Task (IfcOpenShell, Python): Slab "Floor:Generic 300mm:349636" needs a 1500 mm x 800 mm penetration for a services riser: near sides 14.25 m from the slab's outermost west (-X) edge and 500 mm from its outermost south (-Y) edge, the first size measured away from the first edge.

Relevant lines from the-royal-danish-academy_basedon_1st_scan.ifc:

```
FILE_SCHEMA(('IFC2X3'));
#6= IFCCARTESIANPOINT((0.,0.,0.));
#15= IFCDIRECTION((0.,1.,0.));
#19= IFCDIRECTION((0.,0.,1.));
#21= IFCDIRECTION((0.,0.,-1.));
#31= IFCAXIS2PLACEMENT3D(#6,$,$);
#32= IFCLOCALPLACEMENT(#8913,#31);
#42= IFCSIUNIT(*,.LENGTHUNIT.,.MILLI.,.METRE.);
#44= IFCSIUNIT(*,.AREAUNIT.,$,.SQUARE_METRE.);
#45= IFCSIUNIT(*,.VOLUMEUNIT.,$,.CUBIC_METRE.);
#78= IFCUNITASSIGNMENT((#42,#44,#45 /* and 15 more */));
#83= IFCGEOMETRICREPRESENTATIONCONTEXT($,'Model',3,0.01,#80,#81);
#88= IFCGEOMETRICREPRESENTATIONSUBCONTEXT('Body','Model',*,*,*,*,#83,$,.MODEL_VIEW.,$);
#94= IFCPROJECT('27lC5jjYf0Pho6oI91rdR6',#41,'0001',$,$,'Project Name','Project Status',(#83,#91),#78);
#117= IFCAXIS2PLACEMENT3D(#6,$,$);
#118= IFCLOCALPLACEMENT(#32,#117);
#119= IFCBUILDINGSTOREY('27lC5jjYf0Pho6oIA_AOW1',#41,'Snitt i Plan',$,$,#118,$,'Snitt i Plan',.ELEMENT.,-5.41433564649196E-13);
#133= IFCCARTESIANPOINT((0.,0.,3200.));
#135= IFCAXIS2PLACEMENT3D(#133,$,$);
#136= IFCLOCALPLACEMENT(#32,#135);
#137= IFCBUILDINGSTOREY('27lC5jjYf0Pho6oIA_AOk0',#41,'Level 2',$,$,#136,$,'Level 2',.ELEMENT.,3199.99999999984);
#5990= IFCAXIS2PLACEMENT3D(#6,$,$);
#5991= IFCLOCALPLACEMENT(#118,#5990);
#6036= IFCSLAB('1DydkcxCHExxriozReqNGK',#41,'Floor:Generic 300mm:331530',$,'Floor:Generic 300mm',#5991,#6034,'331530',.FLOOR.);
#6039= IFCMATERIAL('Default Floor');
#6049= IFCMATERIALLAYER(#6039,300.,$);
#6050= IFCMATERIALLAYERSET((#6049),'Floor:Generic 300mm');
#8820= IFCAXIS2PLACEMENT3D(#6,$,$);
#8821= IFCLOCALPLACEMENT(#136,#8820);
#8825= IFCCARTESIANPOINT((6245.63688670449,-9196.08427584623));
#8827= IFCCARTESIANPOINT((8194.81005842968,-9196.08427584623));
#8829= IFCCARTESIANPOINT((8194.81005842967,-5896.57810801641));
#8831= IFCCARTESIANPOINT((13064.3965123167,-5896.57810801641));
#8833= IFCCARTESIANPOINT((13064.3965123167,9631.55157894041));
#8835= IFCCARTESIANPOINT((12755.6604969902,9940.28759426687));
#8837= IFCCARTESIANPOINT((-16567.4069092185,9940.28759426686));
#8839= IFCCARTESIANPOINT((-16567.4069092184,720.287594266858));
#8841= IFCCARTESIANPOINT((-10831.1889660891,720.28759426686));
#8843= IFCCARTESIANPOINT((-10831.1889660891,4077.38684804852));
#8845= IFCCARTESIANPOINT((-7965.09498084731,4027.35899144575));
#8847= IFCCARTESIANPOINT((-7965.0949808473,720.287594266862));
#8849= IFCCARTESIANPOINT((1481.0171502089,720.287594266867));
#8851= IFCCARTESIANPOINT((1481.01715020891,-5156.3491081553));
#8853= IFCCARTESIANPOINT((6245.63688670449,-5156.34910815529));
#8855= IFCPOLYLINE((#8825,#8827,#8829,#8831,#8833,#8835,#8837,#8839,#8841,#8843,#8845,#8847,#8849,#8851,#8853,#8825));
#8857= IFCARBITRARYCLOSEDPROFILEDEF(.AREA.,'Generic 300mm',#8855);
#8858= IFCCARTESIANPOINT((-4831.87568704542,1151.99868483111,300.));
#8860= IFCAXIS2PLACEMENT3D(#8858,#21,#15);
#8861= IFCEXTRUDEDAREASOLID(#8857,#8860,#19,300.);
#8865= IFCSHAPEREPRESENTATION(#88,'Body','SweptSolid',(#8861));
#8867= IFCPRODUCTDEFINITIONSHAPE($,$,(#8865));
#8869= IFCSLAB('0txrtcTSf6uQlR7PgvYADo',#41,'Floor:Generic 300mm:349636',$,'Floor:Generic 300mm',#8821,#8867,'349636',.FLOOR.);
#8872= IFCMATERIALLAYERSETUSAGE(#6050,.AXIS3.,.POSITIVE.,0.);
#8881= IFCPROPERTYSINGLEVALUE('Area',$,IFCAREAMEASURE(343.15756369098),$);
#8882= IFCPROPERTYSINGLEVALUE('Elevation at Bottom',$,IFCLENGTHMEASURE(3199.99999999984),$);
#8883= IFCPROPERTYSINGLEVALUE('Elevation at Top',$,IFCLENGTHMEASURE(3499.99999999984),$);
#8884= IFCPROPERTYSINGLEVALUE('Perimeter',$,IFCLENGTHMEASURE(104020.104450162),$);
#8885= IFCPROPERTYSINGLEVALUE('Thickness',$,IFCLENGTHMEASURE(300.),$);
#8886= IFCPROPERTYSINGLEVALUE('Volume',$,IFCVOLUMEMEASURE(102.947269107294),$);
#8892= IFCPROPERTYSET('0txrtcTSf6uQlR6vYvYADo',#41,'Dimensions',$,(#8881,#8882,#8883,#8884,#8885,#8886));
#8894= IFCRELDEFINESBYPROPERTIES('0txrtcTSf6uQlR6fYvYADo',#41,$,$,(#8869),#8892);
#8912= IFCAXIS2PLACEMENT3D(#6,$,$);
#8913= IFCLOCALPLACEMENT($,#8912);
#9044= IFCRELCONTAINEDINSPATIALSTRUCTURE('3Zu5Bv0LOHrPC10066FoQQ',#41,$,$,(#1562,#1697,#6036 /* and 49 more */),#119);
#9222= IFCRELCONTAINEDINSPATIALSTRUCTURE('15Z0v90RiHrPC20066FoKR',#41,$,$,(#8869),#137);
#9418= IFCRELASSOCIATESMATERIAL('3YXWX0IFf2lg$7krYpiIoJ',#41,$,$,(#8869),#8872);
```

```python
import numpy as np
import ifcopenshell
import ifcopenshell.api.feature
import ifcopenshell.api.geometry
import ifcopenshell.api.pset
import ifcopenshell.api.root
import ifcopenshell.geom
import ifcopenshell.util.element
import ifcopenshell.util.placement
import ifcopenshell.util.representation
import ifcopenshell.util.shape
import ifcopenshell.util.unit

model = ifcopenshell.open("the-royal-danish-academy_basedon_1st_scan.ifc")
unit_scale = ifcopenshell.util.unit.calculate_unit_scale(model)
area_scale = ifcopenshell.util.unit.calculate_unit_scale(model, "AREAUNIT")
volume_scale = ifcopenshell.util.unit.calculate_unit_scale(model, "VOLUMEUNIT")
settings = ifcopenshell.geom.settings()


def volume(element):
    """Net volume in cubic metres, openings subtracted."""
    shape = ifcopenshell.geom.create_shape(settings, element)
    return ifcopenshell.util.shape.get_volume(shape.geometry)


slab = model.by_guid("0txrtcTSf6uQlR7PgvYADo")
before = volume(slab)

# Extent in the slab's own axes, in metres. The edges named are its -X and -Y sides.
slab_shape = ifcopenshell.geom.create_shape(settings, slab)
vertices = ifcopenshell.util.shape.get_vertices(slab_shape.geometry)
x_min, y_min, bottom = vertices.min(axis=0)
top = vertices[:, 2].max()

opening = ifcopenshell.api.root.create_entity(model, ifc_class="IfcOpeningElement", name="Services riser opening")
context = ifcopenshell.util.representation.get_context(model, "Model", "Body", "MODEL_VIEW")
width, depth = 1.5, 0.8
outline = [(0.0, 0.0), (width, 0.0), (width, depth), (0.0, depth), (0.0, 0.0)]
# Overshoot both faces by 50 mm so the cut is clean.
shape = ifcopenshell.api.geometry.add_slab_representation(
    model, context=context, depth=top - bottom + 0.1, polyline=outline
)
ifcopenshell.api.geometry.assign_representation(model, product=opening, representation=shape)

matrix = ifcopenshell.util.placement.get_local_placement(slab.ObjectPlacement)
matrix[:, 3] = matrix @ np.append(np.array([x_min + 14.25, y_min + 0.5, bottom - 0.05]) / unit_scale, 1.0)
ifcopenshell.api.geometry.edit_object_placement(model, product=opening, matrix=matrix, is_si=False)
ifcopenshell.api.feature.add_feature(model, feature=opening, element=slab)

after = volume(slab)

# Update the slab's stored quantities.
pset = model.by_id(ifcopenshell.util.element.get_pset(slab, "Dimensions", should_inherit=False)["id"])
ifcopenshell.api.pset.edit_pset(model, pset=pset, properties={
    "Area": model.create_entity("IfcAreaMeasure", after / (top - bottom) / area_scale),
    "Volume": model.create_entity("IfcVolumeMeasure", after / volume_scale),
})

print(f"slab volume {before:.3f} -> {after:.3f} m3")

model.write("the-royal-danish-academy_basedon_1st_scan_updated.ifc")
```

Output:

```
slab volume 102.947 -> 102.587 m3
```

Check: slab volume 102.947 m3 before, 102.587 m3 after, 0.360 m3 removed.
